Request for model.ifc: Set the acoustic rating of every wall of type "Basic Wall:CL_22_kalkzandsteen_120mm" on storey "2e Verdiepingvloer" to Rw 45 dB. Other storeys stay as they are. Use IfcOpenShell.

First a look at what the model holds.

```python
import ifcopenshell
import ifcopenshell.util.element

model = ifcopenshell.open("model.ifc")
print(model.schema)
storey = next(s for s in model.by_type("IfcBuildingStorey") if s.Name == "2e Verdiepingvloer")
walls = [e for e in ifcopenshell.util.element.get_decomposition(storey) if e.is_a("IfcWall")]
seen = {}
for e in walls:
    element_type = ifcopenshell.util.element.get_type(e)
    key = (element_type.Name if element_type != e and element_type else None, ifcopenshell.util.element.get_pset(e, "Pset_WallCommon", "AcousticRating"))
    seen[key] = seen.get(key, 0) + 1
for (name, value), count in sorted(seen.items(), key=str):
    print(count, "x", name, "|", value)
```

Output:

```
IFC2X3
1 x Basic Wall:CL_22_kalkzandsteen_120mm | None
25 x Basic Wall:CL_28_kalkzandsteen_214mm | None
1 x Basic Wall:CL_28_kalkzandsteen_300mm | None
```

```python
import ifcopenshell
import ifcopenshell.api.pset
import ifcopenshell.util.element

model = ifcopenshell.open("model.ifc")

storey = next(s for s in model.by_type("IfcBuildingStorey") if s.Name == "2e Verdiepingvloer")
walls = [e for e in ifcopenshell.util.element.get_decomposition(storey) if e.is_a("IfcWall")]

count = 0
for e in walls:
    element_type = ifcopenshell.util.element.get_type(e)
    if element_type in (None, e) or element_type.Name != "Basic Wall:CL_22_kalkzandsteen_120mm":
        continue
    # add_pset returns the element's existing set when there is one.
    pset = ifcopenshell.api.pset.add_pset(model, product=e, name="Pset_WallCommon")
    ifcopenshell.api.pset.edit_pset(model, pset=pset, properties={"AcousticRating": "Rw 45 dB"})
    count += 1

print(count, "walls updated")

model.write("model_v2.ifc")
```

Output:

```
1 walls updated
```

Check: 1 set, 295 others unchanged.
